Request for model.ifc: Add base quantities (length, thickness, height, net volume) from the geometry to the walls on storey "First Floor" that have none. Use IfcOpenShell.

First a look at what the model holds.

```python
import ifcopenshell
import ifcopenshell.util.element
import ifcopenshell.util.unit

model = ifcopenshell.open("model.ifc")
print(model.schema)
for unit_type in ("LENGTHUNIT", "AREAUNIT", "VOLUMEUNIT"):
    print(unit_type, ifcopenshell.util.unit.calculate_unit_scale(model, unit_type))
storey = next(s for s in model.by_type("IfcBuildingStorey") if s.Name == "First Floor")
walls = [e for e in ifcopenshell.util.element.get_decomposition(storey) if e.is_a("IfcWall")]
for e in sorted(walls, key=lambda e: e.id()):
    print(e.id(), e.is_a(), e.Name, list(ifcopenshell.util.element.get_psets(e, qtos_only=True)), sep=" | ")
```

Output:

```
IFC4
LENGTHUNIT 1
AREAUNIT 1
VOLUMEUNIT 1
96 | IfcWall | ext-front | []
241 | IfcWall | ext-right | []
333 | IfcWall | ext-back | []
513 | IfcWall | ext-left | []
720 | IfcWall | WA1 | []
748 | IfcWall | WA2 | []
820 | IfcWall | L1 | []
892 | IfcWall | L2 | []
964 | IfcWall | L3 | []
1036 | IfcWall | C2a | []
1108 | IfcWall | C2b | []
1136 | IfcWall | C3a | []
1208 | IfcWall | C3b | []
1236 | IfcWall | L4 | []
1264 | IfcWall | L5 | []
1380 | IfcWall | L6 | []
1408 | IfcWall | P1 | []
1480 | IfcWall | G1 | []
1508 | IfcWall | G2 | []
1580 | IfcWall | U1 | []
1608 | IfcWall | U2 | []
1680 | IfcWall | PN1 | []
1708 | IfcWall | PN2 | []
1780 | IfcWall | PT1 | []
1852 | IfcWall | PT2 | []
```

```python
import ifcopenshell
import ifcopenshell.api.pset
import ifcopenshell.geom
import ifcopenshell.util.element
import ifcopenshell.util.shape
import ifcopenshell.util.unit

model = ifcopenshell.open("model.ifc")
unit_scale = ifcopenshell.util.unit.calculate_unit_scale(model)
volume_scale = ifcopenshell.util.unit.calculate_unit_scale(model, "VOLUMEUNIT")
settings = ifcopenshell.geom.settings()

storey = next(s for s in model.by_type("IfcBuildingStorey") if s.Name == "First Floor")
walls = [e for e in ifcopenshell.util.element.get_decomposition(storey) if e.is_a("IfcWall")]

for e in sorted(walls, key=lambda e: e.id()):
    if ifcopenshell.util.element.get_psets(e, qtos_only=True, should_inherit=False):
        continue
    # Geometry comes back in metres, in the element's own axes.
    shape = ifcopenshell.geom.create_shape(settings, e)
    values = {
        "Length": ifcopenshell.util.shape.get_x(shape.geometry) / unit_scale,
        "Width": ifcopenshell.util.shape.get_y(shape.geometry) / unit_scale,
        "Height": ifcopenshell.util.shape.get_z(shape.geometry) / unit_scale,
        "NetVolume": ifcopenshell.util.shape.get_volume(shape.geometry) / volume_scale,
    }
    qto = ifcopenshell.api.pset.add_qto(model, product=e, name="Qto_WallBaseQuantities")
    ifcopenshell.api.pset.edit_qto(model, qto=qto, properties=values)
    print(e.id(), {k: round(v, 3) for k, v in values.items()})

model.write("model_edited.ifc")
```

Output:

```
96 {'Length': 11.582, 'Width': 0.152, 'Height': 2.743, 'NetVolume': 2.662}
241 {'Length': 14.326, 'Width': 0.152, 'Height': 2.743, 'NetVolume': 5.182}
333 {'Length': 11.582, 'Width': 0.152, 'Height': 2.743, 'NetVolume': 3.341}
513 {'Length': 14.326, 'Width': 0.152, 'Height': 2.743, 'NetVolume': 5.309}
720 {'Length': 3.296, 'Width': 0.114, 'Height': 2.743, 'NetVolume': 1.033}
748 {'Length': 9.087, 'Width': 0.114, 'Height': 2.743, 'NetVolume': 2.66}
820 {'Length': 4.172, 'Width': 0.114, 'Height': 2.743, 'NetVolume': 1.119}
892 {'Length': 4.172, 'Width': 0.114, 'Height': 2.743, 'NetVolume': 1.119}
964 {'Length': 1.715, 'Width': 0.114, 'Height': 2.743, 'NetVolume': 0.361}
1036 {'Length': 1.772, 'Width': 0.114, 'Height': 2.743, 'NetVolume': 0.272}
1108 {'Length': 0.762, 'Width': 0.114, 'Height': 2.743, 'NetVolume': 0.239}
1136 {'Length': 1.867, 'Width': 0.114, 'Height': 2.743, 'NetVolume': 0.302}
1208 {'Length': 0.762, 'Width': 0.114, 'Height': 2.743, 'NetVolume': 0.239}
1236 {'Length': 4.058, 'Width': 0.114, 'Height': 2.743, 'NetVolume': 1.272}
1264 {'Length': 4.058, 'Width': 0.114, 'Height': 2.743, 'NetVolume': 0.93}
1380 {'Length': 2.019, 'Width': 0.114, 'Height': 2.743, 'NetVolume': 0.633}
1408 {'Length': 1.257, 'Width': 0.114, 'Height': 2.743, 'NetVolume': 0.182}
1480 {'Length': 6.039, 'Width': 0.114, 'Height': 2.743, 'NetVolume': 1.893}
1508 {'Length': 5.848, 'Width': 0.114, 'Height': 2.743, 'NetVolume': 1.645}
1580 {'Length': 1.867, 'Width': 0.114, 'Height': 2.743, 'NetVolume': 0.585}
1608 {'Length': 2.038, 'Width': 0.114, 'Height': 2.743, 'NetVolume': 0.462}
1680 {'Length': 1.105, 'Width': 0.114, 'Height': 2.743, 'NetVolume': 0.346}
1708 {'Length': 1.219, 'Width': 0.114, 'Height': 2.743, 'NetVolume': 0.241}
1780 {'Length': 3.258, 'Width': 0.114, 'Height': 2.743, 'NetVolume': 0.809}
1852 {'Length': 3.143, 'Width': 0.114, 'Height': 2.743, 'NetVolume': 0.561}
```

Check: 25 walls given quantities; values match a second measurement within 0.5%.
